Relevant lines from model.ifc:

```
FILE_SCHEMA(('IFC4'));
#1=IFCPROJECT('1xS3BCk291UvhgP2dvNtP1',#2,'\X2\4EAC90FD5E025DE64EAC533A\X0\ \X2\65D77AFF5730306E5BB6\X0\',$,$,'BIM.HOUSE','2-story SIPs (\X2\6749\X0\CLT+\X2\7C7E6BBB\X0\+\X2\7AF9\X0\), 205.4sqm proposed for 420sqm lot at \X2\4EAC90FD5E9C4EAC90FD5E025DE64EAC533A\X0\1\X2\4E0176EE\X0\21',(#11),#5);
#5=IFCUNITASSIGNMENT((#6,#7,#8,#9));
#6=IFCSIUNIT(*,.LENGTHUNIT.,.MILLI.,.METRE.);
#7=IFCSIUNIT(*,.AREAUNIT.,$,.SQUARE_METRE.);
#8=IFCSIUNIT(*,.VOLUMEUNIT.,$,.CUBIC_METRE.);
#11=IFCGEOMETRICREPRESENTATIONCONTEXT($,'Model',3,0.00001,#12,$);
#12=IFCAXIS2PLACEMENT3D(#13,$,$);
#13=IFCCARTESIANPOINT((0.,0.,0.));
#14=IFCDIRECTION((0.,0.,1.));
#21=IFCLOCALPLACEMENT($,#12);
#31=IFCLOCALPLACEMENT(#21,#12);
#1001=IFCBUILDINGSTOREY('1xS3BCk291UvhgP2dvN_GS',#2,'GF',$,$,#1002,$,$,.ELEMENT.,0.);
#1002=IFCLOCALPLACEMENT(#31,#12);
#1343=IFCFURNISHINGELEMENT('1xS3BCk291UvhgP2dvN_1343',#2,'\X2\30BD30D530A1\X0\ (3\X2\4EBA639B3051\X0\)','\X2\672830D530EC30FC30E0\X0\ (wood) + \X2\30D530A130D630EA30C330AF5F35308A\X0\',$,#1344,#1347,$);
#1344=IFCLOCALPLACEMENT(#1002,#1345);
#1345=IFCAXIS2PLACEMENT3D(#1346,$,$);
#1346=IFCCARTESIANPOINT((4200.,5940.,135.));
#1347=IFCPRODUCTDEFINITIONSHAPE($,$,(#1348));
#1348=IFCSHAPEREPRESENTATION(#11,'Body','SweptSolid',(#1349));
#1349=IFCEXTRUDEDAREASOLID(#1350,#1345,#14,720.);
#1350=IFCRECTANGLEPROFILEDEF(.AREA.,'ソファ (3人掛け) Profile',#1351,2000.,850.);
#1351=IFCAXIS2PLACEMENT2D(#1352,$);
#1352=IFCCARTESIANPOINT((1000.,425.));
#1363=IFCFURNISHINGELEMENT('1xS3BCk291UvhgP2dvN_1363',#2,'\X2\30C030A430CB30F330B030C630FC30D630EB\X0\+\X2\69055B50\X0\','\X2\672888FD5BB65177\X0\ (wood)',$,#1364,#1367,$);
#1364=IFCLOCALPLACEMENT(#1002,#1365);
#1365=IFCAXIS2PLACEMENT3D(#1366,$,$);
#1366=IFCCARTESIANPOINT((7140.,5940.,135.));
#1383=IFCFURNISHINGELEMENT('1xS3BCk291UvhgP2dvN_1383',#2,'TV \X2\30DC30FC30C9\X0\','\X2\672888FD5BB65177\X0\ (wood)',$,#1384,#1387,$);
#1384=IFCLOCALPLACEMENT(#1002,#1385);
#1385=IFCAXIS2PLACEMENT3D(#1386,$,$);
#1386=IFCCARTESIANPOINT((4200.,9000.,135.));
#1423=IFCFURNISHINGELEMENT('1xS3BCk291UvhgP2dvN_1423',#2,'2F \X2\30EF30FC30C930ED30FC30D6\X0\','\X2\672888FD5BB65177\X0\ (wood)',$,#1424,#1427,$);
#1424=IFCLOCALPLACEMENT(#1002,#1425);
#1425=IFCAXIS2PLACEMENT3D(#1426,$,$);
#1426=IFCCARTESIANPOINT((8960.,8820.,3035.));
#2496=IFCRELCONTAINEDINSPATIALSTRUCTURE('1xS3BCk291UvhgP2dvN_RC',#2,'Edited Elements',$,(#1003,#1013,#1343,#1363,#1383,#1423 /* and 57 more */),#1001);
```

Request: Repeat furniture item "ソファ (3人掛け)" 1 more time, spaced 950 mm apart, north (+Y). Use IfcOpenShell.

```python
import numpy as np
import ifcopenshell
import ifcopenshell.api.geometry
import ifcopenshell.api.root
import ifcopenshell.util.element
import ifcopenshell.util.placement

model = ifcopenshell.open("model.ifc")


def reuse_history(source, copy):
    """copy_class also copies each property set's owner history, people and application; keep the originals."""
    for rel in copy.IsDefinedBy:
        if rel.is_a("IfcRelDefinesByProperties") and (history := rel.RelatingPropertyDefinition.OwnerHistory):
            rel.RelatingPropertyDefinition.OwnerHistory = source.OwnerHistory
            ifcopenshell.util.element.remove_deep2(model, history)


source = model.by_guid("1xS3BCk291UvhgP2dvN_1343")
base = ifcopenshell.util.placement.get_local_placement(source.ObjectPlacement)
step = np.array([0.0, 1.0, 0.0]) * 950.0

for i in range(1, 2):
    copy = ifcopenshell.api.root.copy_class(model, product=source)
    copy.Representation = ifcopenshell.util.element.copy_deep(
        model, source.Representation, exclude=["IfcGeometricRepresentationContext", "IfcRepresentationMap"]
    )
    reuse_history(source, copy)
    matrix = base.copy()
    matrix[:3, 3] += i * step
    print("added at", matrix[:3, 3].round(3) + 0.0)
    ifcopenshell.api.geometry.edit_object_placement(model, product=copy, matrix=matrix, is_si=False)

model.write("model_edited.ifc")
```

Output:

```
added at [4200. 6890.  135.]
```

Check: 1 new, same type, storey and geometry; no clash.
